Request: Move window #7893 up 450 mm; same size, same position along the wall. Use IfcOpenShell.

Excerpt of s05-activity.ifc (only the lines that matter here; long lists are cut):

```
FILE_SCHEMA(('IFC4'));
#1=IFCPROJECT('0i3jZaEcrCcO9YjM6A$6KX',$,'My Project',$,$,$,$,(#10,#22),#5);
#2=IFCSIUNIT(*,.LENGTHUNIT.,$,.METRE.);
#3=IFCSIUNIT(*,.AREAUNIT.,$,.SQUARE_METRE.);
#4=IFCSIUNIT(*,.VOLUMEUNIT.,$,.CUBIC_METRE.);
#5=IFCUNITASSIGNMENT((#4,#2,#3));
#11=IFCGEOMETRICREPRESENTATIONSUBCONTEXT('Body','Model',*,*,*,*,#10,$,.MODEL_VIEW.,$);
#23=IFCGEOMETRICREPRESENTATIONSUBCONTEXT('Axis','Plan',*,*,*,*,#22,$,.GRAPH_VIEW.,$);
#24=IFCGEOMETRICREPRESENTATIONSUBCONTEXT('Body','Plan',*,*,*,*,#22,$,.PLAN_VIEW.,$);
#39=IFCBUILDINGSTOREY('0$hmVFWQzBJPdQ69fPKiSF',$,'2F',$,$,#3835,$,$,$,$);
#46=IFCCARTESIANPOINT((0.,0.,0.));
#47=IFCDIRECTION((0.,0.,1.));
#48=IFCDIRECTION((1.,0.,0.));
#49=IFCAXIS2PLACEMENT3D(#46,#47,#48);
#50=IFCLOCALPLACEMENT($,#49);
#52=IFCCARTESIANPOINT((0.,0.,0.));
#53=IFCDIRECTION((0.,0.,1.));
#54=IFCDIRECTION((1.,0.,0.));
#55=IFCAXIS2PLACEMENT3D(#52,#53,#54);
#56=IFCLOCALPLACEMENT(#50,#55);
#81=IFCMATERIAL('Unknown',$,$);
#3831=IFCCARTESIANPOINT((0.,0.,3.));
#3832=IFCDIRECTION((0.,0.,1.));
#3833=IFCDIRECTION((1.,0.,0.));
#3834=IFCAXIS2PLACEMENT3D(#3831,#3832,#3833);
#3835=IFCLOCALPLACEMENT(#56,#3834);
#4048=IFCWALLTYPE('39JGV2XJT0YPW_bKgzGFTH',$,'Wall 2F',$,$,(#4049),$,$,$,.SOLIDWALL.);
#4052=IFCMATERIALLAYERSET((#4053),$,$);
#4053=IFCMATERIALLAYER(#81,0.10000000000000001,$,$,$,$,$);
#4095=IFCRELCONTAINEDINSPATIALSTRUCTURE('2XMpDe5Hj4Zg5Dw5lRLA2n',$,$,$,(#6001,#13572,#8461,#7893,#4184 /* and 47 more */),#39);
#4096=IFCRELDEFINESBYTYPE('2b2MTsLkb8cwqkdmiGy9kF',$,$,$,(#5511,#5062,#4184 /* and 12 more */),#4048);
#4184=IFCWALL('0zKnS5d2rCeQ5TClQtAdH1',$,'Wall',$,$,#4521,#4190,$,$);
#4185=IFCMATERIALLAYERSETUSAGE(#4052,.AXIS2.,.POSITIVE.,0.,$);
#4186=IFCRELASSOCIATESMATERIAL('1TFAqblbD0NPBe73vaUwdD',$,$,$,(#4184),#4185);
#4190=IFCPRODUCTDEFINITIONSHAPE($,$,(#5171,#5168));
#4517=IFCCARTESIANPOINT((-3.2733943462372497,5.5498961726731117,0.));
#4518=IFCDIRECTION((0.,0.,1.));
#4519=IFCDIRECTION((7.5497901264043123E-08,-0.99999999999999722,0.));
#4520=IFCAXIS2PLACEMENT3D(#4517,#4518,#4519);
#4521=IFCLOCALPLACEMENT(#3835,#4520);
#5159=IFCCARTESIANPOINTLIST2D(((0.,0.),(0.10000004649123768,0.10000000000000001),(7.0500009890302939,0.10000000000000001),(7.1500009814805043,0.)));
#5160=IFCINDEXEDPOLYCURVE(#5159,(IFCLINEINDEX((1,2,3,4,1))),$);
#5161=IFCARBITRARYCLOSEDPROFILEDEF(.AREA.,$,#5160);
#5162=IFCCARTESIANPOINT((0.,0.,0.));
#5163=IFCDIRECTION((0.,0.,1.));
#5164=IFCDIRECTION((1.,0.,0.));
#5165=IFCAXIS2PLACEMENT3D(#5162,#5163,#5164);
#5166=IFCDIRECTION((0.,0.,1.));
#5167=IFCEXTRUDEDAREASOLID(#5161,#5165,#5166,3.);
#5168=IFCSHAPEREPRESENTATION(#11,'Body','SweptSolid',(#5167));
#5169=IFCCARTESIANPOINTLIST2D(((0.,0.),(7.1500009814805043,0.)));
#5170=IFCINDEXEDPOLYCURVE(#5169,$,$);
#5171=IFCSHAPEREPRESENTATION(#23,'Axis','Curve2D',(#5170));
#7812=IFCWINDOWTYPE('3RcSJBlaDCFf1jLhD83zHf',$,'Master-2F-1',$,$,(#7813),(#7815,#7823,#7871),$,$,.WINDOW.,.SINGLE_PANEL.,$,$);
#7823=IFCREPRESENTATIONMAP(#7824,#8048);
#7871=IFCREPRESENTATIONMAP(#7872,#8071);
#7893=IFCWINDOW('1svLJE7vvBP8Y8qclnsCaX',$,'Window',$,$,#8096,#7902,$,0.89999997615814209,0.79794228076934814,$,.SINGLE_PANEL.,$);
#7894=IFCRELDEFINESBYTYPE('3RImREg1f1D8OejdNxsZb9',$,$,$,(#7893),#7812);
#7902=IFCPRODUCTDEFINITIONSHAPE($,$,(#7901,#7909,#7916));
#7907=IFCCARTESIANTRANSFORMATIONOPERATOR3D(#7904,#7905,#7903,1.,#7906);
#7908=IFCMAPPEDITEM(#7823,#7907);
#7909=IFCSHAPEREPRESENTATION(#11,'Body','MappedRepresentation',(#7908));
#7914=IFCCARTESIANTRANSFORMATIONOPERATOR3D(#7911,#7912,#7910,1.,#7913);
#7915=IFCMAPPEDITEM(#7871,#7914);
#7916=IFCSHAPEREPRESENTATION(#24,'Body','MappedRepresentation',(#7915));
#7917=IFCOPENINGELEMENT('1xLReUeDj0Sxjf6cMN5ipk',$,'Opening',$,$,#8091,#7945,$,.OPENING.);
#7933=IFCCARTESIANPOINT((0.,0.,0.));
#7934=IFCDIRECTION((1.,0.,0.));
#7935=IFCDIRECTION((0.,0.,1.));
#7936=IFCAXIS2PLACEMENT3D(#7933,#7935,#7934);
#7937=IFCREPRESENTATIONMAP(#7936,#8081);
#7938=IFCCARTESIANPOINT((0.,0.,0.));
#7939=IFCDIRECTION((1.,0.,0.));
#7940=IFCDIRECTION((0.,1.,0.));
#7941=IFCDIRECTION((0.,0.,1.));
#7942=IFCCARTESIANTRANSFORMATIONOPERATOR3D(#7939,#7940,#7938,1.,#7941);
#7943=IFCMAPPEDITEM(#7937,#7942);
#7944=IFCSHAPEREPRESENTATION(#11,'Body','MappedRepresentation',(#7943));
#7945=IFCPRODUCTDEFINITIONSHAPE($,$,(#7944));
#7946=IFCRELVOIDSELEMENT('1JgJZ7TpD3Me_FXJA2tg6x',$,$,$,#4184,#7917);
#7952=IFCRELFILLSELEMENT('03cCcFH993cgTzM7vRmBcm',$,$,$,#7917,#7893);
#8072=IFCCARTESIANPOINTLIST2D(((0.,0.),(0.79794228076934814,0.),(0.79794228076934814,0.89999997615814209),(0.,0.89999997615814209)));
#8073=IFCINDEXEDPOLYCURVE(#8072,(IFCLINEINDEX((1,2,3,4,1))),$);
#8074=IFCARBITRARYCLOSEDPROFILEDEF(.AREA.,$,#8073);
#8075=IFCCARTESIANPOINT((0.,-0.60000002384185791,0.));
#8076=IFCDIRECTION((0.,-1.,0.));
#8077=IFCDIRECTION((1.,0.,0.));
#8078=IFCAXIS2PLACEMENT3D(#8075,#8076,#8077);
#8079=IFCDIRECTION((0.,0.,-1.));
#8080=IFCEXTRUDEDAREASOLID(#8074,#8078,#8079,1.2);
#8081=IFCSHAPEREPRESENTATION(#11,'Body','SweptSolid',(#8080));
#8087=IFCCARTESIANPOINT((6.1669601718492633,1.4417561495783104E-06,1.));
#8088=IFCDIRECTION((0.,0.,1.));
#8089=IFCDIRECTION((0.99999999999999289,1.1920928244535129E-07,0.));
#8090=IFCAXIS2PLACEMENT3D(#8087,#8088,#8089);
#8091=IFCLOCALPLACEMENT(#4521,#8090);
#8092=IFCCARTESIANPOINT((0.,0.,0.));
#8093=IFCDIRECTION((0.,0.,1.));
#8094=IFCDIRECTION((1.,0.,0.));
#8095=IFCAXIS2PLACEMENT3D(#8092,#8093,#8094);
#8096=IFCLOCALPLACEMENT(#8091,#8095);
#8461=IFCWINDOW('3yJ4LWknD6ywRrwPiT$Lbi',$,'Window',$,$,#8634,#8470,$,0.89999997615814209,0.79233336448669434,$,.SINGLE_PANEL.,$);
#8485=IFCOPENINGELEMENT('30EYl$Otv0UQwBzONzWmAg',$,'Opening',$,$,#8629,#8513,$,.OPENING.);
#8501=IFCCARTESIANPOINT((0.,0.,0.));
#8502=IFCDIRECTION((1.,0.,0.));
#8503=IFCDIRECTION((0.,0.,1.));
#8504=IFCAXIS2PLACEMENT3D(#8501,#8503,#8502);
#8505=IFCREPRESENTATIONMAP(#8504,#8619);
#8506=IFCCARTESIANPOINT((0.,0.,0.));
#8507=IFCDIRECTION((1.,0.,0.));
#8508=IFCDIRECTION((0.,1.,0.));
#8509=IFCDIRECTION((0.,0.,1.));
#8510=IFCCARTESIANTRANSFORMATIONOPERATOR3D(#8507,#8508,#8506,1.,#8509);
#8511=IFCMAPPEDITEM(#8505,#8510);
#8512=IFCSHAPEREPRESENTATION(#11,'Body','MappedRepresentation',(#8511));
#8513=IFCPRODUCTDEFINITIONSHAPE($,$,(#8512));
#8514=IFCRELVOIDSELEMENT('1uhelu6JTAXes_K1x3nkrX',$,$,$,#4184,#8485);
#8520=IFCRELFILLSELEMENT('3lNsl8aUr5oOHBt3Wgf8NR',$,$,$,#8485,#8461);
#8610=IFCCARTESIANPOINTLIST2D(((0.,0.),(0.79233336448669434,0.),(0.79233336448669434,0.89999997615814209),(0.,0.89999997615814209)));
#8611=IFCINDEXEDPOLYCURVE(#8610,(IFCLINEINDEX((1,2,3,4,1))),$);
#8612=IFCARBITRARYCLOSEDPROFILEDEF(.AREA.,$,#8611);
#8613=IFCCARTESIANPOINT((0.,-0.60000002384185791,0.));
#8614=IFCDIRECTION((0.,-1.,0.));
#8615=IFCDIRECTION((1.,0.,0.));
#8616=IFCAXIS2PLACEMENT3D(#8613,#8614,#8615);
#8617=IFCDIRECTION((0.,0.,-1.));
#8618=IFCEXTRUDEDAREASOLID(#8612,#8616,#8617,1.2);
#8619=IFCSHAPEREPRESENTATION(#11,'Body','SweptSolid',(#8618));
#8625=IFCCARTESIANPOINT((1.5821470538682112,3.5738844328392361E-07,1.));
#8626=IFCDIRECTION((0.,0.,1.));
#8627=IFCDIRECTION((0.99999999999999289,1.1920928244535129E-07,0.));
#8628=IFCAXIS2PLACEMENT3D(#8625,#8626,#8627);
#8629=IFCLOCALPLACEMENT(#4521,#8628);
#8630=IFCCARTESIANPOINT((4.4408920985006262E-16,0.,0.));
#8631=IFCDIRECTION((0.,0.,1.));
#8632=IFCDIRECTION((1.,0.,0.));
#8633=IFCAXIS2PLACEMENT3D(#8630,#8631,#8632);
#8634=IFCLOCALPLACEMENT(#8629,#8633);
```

```python
import numpy as np
import ifcopenshell
import ifcopenshell.api.geometry
import ifcopenshell.util.placement
import ifcopenshell.util.unit

model = ifcopenshell.open("s05-activity.ifc")
unit_scale = ifcopenshell.util.unit.calculate_unit_scale(model)

window = model.by_guid("1svLJE7vvBP8Y8qclnsCaX")
opening = window.FillsVoids[0].RelatingOpeningElement
dz = 0.45

shift = np.array([0.0, 0.0, dz])
# The window is placed relative to its opening, so it follows when the opening moves.
matrix = ifcopenshell.util.placement.get_local_placement(opening.ObjectPlacement)
matrix[:3, 3] += shift
ifcopenshell.api.geometry.edit_object_placement(
    model, product=opening, matrix=matrix, is_si=False, should_transform_children=True
)

print(f"moved by {dz * unit_scale:+.3f} m")

model.write("s05-activity_updated.ifc")
```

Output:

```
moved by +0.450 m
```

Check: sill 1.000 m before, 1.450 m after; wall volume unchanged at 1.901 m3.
